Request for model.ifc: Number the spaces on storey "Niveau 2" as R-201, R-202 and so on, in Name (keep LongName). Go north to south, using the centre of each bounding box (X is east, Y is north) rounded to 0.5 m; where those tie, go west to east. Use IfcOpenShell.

First a look at what the model holds.

```python
import ifcopenshell
import ifcopenshell.util.element
import ifcopenshell.util.placement

model = ifcopenshell.open("model.ifc")
print(model.schema)
storey = next(s for s in model.by_type("IfcBuildingStorey") if s.Name == "Niveau 2")
spaces = [e for e in ifcopenshell.util.element.get_decomposition(storey) if e.is_a("IfcSpace")]
for e in sorted(spaces, key=lambda e: e.id()):
    origin = ifcopenshell.util.placement.get_local_placement(e.ObjectPlacement)[:3, 3]
    print(e.id(), e.Name, e.LongName, origin.round(2) + 0.0, sep=" | ")
```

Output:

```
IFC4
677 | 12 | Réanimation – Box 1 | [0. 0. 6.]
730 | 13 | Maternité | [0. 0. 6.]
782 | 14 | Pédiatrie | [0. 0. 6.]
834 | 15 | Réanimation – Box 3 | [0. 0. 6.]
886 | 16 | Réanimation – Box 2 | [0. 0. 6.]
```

```python
import ifcopenshell
import ifcopenshell.geom
import ifcopenshell.util.element
import ifcopenshell.util.shape

model = ifcopenshell.open("model.ifc")
settings = ifcopenshell.geom.settings()
settings.set("use-world-coords", True)


def centre(element):
    shape = ifcopenshell.geom.create_shape(settings, element)
    return ifcopenshell.util.shape.get_bbox_centroid(shape.geometry)


storey = next(s for s in model.by_type("IfcBuildingStorey") if s.Name == "Niveau 2")
spaces = [e for e in ifcopenshell.util.element.get_decomposition(storey) if e.is_a("IfcSpace")]

# Insertion points can sit at a corner or the storey origin, so sort by the geometry (in metres).
centres = {e: centre(e) for e in spaces}
spaces.sort(key=lambda e: (-round(centres[e][1] / 0.5), centres[e][0]))

for i, e in enumerate(spaces, start=1):
    number = f"R-2{i:02d}"
    e.Name = number
    print(e.id(), number)

model.write("model_v2.ifc")
```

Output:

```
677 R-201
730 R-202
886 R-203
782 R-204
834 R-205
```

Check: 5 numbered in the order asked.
